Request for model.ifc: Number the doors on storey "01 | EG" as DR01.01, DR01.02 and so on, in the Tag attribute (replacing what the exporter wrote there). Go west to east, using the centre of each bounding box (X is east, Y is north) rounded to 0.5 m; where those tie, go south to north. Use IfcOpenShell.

First a look at what the model holds.

```python
import ifcopenshell
import ifcopenshell.util.element
import ifcopenshell.util.placement

model = ifcopenshell.open("model.ifc")
print(model.schema)
storey = next(s for s in model.by_type("IfcBuildingStorey") if s.Name == "01 | EG")
doors = [e for e in ifcopenshell.util.element.get_decomposition(storey) if e.is_a("IfcDoor")]
for e in sorted(doors, key=lambda e: e.id()):
    origin = ifcopenshell.util.placement.get_local_placement(e.ObjectPlacement)[:3, 3]
    print(e.id(), e.Tag, e.Name, origin.round(2) + 0.0, sep=" | ")
```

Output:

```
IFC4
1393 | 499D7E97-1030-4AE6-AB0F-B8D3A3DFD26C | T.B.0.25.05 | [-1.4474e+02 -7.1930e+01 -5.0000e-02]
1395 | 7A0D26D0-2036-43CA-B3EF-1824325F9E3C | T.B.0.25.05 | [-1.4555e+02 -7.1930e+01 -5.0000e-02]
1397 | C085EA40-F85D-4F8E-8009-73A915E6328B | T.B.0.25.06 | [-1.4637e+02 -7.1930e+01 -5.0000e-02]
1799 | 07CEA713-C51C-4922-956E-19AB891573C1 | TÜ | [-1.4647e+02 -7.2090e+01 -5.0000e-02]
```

```python
import ifcopenshell
import ifcopenshell.geom
import ifcopenshell.util.element
import ifcopenshell.util.shape

model = ifcopenshell.open("model.ifc")
settings = ifcopenshell.geom.settings()
settings.set("use-world-coords", True)


def centre(element):
    shape = ifcopenshell.geom.create_shape(settings, element)
    return ifcopenshell.util.shape.get_bbox_centroid(shape.geometry)


storey = next(s for s in model.by_type("IfcBuildingStorey") if s.Name == "01 | EG")
doors = [e for e in ifcopenshell.util.element.get_decomposition(storey) if e.is_a("IfcDoor")]

# Insertion points can sit at a corner or the storey origin, so sort by the geometry (in metres).
centres = {e: centre(e) for e in doors}
doors.sort(key=lambda e: (round(centres[e][0] / 0.5), centres[e][1]))

for i, e in enumerate(doors, start=1):
    number = f"DR01.{i:02d}"
    e.Tag = number
    print(e.id(), number)

model.write("model_edited.ifc")
```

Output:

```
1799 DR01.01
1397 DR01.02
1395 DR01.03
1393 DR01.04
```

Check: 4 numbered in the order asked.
